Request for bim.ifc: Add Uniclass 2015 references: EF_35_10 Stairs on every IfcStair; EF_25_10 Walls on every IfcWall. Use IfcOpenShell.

First a look at what the model holds.

```python
import ifcopenshell

model = ifcopenshell.open("bim.ifc")
print(model.schema)
print("classifications:", [c.Name for c in model.by_type("IfcClassification")])
for ifc_class in ("IfcDoor", "IfcRoof", "IfcStair", "IfcWall", "IfcWindow"):
    print(ifc_class, len(model.by_type(ifc_class)))
```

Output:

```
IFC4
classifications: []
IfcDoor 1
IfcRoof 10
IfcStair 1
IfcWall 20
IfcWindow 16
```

```python
import ifcopenshell
import ifcopenshell.api.classification

model = ifcopenshell.open("bim.ifc")

system = ifcopenshell.api.classification.add_classification(model, classification="Uniclass 2015")

codes = {
    "IfcStair": ("EF_35_10", "Stairs"),
    "IfcWall": ("EF_25_10", "Walls"),
}
for ifc_class, (code, name) in codes.items():
    products = model.by_type(ifc_class)
    ifcopenshell.api.classification.add_reference(
        model, products=products, classification=system, identification=code, name=name
    )
    print(code, len(products))

model.write("bim_edited.ifc")
```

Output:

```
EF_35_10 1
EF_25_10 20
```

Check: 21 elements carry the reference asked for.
